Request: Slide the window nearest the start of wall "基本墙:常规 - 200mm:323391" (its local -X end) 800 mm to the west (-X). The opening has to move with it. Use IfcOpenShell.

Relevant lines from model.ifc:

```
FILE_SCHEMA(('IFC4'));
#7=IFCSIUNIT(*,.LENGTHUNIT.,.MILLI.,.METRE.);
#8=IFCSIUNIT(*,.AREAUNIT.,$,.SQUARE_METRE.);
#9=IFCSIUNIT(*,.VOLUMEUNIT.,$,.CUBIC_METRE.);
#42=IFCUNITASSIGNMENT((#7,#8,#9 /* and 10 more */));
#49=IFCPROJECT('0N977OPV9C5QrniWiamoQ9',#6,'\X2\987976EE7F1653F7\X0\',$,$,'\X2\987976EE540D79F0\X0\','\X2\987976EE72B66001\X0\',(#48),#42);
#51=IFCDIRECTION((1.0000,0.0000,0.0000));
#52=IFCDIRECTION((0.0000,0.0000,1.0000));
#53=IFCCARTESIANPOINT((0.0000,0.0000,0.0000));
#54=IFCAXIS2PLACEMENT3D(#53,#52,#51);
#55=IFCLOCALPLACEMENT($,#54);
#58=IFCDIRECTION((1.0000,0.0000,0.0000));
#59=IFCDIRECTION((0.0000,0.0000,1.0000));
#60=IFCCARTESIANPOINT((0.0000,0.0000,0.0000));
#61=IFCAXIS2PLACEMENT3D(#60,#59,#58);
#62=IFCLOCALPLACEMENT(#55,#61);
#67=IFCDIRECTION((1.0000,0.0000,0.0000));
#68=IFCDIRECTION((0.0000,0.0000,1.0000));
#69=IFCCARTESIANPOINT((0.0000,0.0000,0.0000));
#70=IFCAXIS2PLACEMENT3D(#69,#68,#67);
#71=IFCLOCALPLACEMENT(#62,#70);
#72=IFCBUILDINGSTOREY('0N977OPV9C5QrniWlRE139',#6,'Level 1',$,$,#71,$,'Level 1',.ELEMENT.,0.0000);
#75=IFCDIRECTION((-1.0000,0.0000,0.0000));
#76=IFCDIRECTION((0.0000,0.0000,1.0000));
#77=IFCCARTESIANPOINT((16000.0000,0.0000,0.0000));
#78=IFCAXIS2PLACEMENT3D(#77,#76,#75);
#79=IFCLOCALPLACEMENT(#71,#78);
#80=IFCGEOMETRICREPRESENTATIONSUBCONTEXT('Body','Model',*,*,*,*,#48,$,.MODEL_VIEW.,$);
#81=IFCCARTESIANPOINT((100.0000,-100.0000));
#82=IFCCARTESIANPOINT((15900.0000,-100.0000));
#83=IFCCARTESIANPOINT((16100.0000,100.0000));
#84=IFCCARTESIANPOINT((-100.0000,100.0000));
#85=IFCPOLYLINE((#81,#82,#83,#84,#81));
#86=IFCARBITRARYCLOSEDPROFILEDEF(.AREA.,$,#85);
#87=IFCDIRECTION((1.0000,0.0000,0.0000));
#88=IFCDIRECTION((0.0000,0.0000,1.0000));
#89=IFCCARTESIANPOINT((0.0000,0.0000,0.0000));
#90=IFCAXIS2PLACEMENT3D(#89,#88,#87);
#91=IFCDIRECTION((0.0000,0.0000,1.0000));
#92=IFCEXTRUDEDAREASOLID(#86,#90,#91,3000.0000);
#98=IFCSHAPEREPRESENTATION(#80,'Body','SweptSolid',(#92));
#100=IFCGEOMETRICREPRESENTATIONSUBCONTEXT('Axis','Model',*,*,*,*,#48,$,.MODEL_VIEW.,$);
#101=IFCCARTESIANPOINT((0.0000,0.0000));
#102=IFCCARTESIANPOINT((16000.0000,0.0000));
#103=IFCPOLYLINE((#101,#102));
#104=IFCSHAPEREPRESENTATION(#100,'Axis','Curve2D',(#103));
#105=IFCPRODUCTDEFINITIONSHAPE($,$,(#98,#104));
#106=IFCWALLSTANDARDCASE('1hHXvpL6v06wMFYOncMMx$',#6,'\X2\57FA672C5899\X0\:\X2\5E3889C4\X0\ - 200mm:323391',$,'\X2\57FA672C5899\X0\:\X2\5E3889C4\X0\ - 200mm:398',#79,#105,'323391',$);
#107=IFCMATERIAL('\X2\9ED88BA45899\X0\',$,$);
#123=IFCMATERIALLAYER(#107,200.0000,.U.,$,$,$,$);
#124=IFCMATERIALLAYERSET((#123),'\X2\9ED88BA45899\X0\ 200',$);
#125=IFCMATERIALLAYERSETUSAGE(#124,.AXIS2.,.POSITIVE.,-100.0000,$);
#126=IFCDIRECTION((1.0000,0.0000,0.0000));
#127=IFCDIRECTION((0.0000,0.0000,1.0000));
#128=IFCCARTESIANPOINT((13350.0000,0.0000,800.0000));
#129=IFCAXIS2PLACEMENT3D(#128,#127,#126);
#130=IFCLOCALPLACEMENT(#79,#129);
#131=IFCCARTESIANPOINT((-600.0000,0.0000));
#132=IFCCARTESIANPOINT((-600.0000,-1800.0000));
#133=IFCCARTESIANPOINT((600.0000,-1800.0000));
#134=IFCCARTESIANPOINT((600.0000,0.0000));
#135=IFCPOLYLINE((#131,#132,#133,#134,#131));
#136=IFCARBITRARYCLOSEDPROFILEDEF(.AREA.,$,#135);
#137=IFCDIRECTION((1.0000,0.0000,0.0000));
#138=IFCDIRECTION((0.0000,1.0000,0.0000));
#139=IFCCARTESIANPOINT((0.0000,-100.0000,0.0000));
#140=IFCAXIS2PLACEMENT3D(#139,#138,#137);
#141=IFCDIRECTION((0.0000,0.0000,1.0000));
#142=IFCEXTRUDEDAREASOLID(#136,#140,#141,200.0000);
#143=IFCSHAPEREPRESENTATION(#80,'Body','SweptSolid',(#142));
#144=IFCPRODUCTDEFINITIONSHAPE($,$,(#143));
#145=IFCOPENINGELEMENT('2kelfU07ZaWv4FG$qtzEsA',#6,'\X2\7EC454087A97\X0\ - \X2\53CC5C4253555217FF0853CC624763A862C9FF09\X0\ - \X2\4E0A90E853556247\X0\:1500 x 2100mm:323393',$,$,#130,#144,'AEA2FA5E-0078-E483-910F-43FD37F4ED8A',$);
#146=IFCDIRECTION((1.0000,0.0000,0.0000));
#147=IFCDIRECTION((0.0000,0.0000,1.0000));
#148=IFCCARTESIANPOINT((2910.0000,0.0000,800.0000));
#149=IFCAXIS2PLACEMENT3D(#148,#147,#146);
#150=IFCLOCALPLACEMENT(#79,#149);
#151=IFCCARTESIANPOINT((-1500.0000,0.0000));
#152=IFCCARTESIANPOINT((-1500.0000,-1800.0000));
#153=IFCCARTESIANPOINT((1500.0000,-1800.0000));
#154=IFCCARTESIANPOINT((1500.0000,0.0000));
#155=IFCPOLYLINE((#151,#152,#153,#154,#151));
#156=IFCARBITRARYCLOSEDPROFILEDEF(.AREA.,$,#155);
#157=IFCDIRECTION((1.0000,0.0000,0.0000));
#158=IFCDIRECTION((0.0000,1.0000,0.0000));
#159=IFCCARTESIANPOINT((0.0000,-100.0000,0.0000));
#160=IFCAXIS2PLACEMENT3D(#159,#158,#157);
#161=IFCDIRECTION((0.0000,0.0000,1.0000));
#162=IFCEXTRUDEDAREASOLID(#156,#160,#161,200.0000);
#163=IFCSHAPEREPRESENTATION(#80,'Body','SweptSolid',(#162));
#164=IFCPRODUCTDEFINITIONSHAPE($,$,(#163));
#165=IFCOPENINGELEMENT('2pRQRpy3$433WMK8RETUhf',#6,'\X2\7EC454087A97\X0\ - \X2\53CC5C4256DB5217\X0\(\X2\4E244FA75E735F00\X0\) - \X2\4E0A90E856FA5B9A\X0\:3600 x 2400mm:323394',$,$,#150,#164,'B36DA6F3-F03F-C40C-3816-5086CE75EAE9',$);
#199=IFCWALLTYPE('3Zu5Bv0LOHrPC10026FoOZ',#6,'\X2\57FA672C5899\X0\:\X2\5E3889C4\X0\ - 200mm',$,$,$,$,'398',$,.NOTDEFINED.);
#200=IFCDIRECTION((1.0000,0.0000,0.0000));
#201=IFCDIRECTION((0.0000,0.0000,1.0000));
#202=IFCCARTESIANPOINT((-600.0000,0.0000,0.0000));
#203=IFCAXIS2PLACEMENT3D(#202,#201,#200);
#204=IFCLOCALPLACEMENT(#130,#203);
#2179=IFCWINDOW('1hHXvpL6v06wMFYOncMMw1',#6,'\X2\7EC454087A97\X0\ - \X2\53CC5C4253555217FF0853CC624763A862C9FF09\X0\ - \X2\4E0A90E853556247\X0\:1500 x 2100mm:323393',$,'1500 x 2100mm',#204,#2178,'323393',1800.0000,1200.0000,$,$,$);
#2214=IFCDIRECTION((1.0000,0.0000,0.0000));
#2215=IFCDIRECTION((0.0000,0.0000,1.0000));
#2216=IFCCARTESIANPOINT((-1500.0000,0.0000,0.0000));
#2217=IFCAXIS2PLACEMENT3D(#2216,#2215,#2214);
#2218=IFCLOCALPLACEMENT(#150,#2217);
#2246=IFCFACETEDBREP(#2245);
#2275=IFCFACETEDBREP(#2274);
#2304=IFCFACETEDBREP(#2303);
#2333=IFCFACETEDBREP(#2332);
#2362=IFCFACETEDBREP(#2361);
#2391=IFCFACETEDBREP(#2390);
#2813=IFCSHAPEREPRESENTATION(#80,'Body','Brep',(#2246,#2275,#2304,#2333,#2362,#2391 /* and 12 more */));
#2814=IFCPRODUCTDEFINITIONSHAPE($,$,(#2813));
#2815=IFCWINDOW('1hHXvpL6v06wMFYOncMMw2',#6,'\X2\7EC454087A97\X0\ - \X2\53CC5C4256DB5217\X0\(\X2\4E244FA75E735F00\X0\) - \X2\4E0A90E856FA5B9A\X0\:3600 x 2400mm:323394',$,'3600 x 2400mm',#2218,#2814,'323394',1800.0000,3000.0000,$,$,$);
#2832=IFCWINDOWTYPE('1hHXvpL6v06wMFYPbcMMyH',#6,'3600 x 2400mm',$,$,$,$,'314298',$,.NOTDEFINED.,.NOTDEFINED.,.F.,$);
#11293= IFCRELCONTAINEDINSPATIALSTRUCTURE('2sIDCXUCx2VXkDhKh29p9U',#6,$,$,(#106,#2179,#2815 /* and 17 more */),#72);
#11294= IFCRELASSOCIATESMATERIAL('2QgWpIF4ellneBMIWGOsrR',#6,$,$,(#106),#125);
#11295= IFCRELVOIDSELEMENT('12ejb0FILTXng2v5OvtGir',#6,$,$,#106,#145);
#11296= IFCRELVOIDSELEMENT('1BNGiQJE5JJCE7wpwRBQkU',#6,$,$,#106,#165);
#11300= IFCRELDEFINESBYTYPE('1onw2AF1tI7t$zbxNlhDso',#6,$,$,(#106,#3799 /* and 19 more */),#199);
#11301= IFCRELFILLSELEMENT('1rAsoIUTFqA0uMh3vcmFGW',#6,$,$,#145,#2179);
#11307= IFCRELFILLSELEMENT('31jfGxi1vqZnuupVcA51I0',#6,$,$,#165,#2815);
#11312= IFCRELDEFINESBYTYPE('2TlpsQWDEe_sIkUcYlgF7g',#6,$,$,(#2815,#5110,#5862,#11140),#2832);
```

```python
import ifcopenshell
import ifcopenshell.api.geometry
import ifcopenshell.util.placement

model = ifcopenshell.open("model.ifc")

window = model.by_id(2815)
opening = window.FillsVoids[0].RelatingOpeningElement
wall = opening.VoidsElements[0].RelatingBuildingElement

wall_matrix = ifcopenshell.util.placement.get_local_placement(wall.ObjectPlacement)
shift = wall_matrix[:3, 0] * 800.0
before = ifcopenshell.util.placement.get_local_placement(window.ObjectPlacement)[:3, 3].copy()

# The window is placed relative to its opening, so it follows when the opening moves.
matrix = ifcopenshell.util.placement.get_local_placement(opening.ObjectPlacement)
matrix[:3, 3] += shift
ifcopenshell.api.geometry.edit_object_placement(
    model, product=opening, matrix=matrix, is_si=False, should_transform_children=True
)

after = ifcopenshell.util.placement.get_local_placement(window.ObjectPlacement)[:3, 3]
print("window moved by", (after - before).round(3) + 0.0)

model.write("model_edited.ifc")
```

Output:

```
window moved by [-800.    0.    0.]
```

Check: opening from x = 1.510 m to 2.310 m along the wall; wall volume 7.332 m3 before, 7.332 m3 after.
